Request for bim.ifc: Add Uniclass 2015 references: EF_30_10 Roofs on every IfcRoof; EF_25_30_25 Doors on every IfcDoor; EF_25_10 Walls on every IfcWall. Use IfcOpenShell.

First a look at what the model holds.

```python
import ifcopenshell

model = ifcopenshell.open("bim.ifc")
print(model.schema)
print("classifications:", [c.Name for c in model.by_type("IfcClassification")])
for ifc_class in ("IfcDoor", "IfcRoof", "IfcStair", "IfcWall", "IfcWindow"):
    print(ifc_class, len(model.by_type(ifc_class)))
```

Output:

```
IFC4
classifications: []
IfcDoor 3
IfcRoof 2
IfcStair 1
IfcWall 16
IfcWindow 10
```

```python
import ifcopenshell
import ifcopenshell.api.classification

model = ifcopenshell.open("bim.ifc")

system = ifcopenshell.api.classification.add_classification(model, classification="Uniclass 2015")

codes = {
    "IfcRoof": ("EF_30_10", "Roofs"),
    "IfcDoor": ("EF_25_30_25", "Doors"),
    "IfcWall": ("EF_25_10", "Walls"),
}
for ifc_class, (code, name) in codes.items():
    products = model.by_type(ifc_class)
    ifcopenshell.api.classification.add_reference(
        model, products=products, classification=system, identification=code, name=name
    )
    print(code, len(products))

model.write("bim_v2.ifc")
```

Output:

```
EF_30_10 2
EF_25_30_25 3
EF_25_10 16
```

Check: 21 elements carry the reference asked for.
